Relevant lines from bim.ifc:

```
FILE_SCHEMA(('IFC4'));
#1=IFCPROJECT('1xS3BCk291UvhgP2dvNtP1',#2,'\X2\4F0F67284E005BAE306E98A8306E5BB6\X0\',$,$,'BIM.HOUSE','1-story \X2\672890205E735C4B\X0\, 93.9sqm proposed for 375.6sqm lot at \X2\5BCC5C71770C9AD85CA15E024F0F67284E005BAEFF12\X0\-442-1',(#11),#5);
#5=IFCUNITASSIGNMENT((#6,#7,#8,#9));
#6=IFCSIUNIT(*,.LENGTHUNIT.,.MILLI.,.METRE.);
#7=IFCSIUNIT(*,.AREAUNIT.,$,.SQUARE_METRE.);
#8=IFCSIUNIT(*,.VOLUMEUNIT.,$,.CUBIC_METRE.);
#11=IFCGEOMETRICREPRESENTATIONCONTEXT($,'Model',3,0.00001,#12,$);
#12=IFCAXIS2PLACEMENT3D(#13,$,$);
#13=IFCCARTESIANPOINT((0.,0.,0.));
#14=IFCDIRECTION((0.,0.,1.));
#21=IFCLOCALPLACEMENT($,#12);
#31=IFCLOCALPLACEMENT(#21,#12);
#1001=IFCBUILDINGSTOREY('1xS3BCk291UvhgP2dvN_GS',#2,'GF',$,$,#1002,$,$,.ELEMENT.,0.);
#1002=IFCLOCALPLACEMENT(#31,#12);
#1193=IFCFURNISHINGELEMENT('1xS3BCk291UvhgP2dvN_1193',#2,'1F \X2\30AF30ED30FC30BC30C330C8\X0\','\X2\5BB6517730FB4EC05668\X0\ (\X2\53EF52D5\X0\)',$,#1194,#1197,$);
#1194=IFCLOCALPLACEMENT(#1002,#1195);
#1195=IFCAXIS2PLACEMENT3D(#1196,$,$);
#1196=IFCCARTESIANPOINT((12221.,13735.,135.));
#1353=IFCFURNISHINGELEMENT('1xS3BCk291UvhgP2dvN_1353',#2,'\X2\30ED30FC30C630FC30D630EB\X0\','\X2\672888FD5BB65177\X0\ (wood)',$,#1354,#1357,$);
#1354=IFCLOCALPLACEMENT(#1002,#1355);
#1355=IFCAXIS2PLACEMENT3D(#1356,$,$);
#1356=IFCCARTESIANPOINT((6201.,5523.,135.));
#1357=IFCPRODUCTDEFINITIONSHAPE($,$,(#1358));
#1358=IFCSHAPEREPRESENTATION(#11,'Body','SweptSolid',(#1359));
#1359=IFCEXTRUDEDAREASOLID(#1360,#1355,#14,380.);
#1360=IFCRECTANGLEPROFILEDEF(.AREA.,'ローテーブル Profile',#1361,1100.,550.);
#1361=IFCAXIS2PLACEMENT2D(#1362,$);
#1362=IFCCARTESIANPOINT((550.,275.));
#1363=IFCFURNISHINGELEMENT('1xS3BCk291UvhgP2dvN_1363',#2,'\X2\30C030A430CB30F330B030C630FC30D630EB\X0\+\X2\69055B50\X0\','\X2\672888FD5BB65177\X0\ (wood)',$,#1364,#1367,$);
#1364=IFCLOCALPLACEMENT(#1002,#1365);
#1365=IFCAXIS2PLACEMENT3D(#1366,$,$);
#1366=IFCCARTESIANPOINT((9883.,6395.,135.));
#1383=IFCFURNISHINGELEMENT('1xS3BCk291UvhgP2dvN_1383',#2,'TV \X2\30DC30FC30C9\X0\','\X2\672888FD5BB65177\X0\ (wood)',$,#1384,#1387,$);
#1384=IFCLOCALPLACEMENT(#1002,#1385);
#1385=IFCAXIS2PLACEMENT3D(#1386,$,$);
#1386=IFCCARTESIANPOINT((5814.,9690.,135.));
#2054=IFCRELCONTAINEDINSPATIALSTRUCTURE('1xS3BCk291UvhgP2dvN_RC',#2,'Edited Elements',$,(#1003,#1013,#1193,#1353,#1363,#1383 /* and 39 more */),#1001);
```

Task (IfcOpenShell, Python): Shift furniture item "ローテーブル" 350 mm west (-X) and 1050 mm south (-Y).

```python
import ifcopenshell
import ifcopenshell.api.geometry
import ifcopenshell.util.placement

model = ifcopenshell.open("bim.ifc")

item = model.by_guid("1xS3BCk291UvhgP2dvN_1353")
matrix = ifcopenshell.util.placement.get_local_placement(item.ObjectPlacement)
matrix[0, 3] -= 350.0
matrix[1, 3] -= 1050.0
ifcopenshell.api.geometry.edit_object_placement(model, product=item, matrix=matrix, is_si=False)

print(ifcopenshell.util.placement.get_local_placement(item.ObjectPlacement).round(3) + 0.0)

model.write("bim-out.ifc")
```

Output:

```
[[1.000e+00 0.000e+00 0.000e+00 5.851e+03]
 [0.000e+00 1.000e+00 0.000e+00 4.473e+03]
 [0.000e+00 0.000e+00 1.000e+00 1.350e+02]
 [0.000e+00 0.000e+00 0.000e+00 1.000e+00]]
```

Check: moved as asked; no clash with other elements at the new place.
